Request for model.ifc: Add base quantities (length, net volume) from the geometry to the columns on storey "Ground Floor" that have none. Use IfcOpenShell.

First a look at what the model holds.

```python
import ifcopenshell
import ifcopenshell.util.element
import ifcopenshell.util.unit

model = ifcopenshell.open("model.ifc")
print(model.schema)
for unit_type in ("LENGTHUNIT", "AREAUNIT", "VOLUMEUNIT"):
    print(unit_type, ifcopenshell.util.unit.calculate_unit_scale(model, unit_type))
storey = next(s for s in model.by_type("IfcBuildingStorey") if s.Name == "Ground Floor")
columns = [e for e in ifcopenshell.util.element.get_decomposition(storey) if e.is_a("IfcColumn")]
for e in sorted(columns, key=lambda e: e.id()):
    print(e.id(), e.is_a(), e.Name, list(ifcopenshell.util.element.get_psets(e, qtos_only=True)), sep=" | ")
```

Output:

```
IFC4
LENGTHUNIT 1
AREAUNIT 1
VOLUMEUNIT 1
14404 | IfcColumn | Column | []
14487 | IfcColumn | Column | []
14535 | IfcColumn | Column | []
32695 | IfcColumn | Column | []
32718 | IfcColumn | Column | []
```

```python
import ifcopenshell
import ifcopenshell.api.pset
import ifcopenshell.geom
import ifcopenshell.util.element
import ifcopenshell.util.shape
import ifcopenshell.util.unit

model = ifcopenshell.open("model.ifc")
unit_scale = ifcopenshell.util.unit.calculate_unit_scale(model)
volume_scale = ifcopenshell.util.unit.calculate_unit_scale(model, "VOLUMEUNIT")
settings = ifcopenshell.geom.settings()

storey = next(s for s in model.by_type("IfcBuildingStorey") if s.Name == "Ground Floor")
columns = [e for e in ifcopenshell.util.element.get_decomposition(storey) if e.is_a("IfcColumn")]

for e in sorted(columns, key=lambda e: e.id()):
    if ifcopenshell.util.element.get_psets(e, qtos_only=True, should_inherit=False):
        continue
    # Geometry comes back in metres, in the element's own axes.
    shape = ifcopenshell.geom.create_shape(settings, e)
    values = {
        "Length": ifcopenshell.util.shape.get_z(shape.geometry) / unit_scale,
        "NetVolume": ifcopenshell.util.shape.get_volume(shape.geometry) / volume_scale,
    }
    qto = ifcopenshell.api.pset.add_qto(model, product=e, name="Qto_ColumnBaseQuantities")
    ifcopenshell.api.pset.edit_qto(model, qto=qto, properties=values)
    print(e.id(), {k: round(v, 3) for k, v in values.items()})

model.write("model_edited.ifc")
```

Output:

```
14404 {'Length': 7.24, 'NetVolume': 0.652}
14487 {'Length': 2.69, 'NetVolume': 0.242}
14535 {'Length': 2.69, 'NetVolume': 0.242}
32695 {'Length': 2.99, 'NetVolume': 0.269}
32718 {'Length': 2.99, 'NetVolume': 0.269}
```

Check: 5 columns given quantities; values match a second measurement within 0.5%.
